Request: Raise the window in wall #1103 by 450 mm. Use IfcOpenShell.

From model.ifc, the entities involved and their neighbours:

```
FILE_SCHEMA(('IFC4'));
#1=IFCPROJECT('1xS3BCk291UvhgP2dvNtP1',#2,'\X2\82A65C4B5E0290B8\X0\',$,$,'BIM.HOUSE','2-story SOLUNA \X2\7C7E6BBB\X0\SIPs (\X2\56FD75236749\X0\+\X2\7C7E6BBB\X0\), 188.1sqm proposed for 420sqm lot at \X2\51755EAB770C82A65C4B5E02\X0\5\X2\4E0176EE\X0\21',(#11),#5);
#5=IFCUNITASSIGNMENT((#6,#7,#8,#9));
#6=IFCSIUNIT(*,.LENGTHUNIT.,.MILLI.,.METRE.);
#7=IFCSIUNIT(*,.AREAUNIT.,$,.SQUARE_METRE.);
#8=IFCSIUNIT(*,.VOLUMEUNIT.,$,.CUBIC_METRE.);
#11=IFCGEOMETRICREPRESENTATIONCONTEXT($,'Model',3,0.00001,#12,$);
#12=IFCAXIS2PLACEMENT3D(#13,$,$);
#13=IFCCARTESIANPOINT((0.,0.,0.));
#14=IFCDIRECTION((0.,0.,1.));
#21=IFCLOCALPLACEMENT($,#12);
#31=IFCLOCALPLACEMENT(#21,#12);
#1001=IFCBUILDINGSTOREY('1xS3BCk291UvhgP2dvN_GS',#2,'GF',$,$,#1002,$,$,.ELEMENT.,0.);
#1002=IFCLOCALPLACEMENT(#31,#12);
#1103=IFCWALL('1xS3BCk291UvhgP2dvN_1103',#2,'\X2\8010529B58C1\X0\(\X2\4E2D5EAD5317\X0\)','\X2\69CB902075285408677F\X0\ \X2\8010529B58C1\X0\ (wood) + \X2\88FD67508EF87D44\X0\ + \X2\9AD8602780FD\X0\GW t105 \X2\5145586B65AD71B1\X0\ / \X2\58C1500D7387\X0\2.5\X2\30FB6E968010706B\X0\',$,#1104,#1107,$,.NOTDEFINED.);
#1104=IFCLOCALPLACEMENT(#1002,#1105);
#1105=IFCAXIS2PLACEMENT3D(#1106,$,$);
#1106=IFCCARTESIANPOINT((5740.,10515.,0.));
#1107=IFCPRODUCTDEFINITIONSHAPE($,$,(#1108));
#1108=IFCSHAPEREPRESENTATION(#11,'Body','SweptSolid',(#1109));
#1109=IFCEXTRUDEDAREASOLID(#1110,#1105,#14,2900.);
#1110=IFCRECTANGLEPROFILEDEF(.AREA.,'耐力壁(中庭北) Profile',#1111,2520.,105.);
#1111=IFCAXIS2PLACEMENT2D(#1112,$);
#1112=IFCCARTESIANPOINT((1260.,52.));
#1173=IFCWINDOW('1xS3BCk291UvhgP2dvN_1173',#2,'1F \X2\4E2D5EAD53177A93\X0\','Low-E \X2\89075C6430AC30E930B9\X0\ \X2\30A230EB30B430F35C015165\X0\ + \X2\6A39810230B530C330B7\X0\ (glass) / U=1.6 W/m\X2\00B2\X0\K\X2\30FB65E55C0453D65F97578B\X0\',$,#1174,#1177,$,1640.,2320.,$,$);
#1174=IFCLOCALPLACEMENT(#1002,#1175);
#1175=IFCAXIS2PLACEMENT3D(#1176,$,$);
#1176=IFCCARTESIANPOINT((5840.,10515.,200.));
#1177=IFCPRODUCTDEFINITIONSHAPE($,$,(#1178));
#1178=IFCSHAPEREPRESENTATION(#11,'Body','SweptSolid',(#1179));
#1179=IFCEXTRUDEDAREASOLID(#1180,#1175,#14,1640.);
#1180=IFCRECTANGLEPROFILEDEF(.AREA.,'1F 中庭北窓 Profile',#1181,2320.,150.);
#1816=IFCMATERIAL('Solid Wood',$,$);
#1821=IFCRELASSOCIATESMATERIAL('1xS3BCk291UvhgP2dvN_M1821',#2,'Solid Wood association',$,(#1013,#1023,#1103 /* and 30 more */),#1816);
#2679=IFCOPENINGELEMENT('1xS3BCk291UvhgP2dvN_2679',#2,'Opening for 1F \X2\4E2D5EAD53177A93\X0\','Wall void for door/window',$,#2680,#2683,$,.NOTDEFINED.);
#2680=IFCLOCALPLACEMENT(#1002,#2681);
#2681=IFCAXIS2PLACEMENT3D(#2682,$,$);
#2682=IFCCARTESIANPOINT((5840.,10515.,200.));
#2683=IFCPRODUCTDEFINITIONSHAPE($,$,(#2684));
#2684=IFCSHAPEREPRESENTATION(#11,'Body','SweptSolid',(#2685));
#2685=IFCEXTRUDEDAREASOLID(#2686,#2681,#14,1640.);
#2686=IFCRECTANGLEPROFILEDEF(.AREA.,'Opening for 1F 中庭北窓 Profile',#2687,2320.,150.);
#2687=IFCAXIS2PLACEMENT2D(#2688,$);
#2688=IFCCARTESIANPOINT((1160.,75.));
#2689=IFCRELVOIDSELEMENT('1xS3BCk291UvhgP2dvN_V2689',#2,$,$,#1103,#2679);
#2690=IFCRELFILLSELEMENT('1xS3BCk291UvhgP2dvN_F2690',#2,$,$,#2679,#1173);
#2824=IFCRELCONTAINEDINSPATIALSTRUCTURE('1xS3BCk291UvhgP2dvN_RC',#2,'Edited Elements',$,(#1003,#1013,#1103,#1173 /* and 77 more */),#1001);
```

```python
import numpy as np
import ifcopenshell
import ifcopenshell.api.geometry
import ifcopenshell.util.placement
import ifcopenshell.util.unit

model = ifcopenshell.open("model.ifc")
unit_scale = ifcopenshell.util.unit.calculate_unit_scale(model)

window = model.by_guid("1xS3BCk291UvhgP2dvN_1173")
opening = window.FillsVoids[0].RelatingOpeningElement
dz = 0.45 / unit_scale

shift = np.array([0.0, 0.0, dz])
# The window is not placed relative to its opening, so move both.
for product in (opening, window):
    matrix = ifcopenshell.util.placement.get_local_placement(product.ObjectPlacement)
    matrix[:3, 3] += shift
    ifcopenshell.api.geometry.edit_object_placement(model, product=product, matrix=matrix, is_si=False)

print(f"moved by {dz * unit_scale:+.3f} m")

model.write("model_edited.ifc")
```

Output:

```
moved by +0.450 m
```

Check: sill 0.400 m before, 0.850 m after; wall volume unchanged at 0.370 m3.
